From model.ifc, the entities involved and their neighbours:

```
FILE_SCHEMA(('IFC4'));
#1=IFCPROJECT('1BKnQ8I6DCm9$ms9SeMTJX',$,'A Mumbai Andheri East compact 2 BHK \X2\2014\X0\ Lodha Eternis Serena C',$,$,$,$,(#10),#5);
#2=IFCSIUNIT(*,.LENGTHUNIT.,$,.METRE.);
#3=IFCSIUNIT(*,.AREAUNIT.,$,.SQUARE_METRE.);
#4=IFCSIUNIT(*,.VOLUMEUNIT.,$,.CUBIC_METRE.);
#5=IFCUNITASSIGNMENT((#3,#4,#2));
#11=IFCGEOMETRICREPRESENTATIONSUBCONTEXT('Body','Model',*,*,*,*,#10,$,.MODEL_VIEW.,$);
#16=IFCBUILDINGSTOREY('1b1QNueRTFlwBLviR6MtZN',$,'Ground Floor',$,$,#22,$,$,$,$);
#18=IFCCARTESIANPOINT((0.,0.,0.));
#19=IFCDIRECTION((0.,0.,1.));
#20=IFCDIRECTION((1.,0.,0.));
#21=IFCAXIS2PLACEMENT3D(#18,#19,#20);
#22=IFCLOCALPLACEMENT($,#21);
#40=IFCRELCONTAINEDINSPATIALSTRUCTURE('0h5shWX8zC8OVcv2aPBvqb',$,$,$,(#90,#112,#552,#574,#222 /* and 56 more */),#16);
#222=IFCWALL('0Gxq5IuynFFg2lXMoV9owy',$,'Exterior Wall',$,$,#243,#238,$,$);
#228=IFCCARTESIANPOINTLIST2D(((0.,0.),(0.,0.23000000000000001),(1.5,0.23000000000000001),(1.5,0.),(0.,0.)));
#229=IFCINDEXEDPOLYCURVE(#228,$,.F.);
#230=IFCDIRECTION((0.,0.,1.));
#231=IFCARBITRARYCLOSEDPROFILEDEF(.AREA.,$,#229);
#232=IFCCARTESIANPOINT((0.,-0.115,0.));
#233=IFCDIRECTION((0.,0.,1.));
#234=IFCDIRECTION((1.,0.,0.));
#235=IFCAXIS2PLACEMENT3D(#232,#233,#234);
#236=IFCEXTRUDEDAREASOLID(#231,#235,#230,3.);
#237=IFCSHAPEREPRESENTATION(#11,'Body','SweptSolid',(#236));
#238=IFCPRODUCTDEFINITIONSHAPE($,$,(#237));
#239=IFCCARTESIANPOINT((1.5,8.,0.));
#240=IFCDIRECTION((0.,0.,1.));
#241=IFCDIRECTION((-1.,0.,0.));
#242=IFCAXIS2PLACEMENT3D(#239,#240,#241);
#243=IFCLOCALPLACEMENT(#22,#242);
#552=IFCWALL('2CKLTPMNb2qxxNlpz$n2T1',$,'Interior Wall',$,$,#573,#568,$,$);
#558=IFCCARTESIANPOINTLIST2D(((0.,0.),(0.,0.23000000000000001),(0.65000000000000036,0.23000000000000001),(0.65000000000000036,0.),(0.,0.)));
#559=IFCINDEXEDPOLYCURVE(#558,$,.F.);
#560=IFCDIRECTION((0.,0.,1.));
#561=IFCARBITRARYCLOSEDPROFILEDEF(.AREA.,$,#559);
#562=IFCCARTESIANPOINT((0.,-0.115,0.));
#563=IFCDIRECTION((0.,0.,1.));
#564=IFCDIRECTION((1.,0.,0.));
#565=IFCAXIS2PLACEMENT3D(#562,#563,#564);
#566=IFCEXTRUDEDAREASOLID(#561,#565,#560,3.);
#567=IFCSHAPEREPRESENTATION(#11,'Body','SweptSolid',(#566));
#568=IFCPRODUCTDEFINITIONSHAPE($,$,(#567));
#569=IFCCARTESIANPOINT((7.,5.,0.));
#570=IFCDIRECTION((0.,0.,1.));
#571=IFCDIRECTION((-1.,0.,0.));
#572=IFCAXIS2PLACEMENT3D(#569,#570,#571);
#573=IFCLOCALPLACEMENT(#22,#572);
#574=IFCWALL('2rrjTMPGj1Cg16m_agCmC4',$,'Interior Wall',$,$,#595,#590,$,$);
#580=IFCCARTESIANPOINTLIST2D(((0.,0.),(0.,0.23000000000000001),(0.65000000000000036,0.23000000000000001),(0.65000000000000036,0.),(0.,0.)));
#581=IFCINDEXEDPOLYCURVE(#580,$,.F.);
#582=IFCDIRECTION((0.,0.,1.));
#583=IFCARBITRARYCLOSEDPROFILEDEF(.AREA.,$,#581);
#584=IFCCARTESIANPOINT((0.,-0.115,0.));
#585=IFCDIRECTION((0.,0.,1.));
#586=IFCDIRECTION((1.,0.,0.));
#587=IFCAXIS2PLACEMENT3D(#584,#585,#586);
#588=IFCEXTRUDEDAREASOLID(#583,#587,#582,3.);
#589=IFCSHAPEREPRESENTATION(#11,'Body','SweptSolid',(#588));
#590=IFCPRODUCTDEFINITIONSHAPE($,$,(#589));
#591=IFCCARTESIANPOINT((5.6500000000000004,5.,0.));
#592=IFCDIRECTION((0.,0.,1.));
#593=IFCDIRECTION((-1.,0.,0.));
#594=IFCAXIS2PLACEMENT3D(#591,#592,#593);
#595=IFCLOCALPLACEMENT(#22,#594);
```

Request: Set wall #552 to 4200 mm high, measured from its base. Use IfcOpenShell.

```python
import ifcopenshell
import ifcopenshell.geom
import ifcopenshell.util.representation
import ifcopenshell.util.shape
import ifcopenshell.util.unit

model = ifcopenshell.open("model.ifc")
unit_scale = ifcopenshell.util.unit.calculate_unit_scale(model)
settings = ifcopenshell.geom.settings()


def volume(element):
    """Net volume in cubic metres, openings subtracted."""
    shape = ifcopenshell.geom.create_shape(settings, element)
    return ifcopenshell.util.shape.get_volume(shape.geometry)


wall = model.by_guid("2CKLTPMNb2qxxNlpz$n2T1")
before = volume(wall)

body = ifcopenshell.util.representation.get_representation(wall, "Model", "Body")
solid = body.Items[0]
old_height = solid.Depth
solid.Depth = 4.2 / unit_scale
after = volume(wall)

print(f"height {old_height:g} -> {solid.Depth:g}, volume {before:.3f} -> {after:.3f} m3")

model.write("model-out.ifc")
```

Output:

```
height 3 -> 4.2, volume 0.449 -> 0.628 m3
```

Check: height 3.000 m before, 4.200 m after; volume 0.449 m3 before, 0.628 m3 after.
